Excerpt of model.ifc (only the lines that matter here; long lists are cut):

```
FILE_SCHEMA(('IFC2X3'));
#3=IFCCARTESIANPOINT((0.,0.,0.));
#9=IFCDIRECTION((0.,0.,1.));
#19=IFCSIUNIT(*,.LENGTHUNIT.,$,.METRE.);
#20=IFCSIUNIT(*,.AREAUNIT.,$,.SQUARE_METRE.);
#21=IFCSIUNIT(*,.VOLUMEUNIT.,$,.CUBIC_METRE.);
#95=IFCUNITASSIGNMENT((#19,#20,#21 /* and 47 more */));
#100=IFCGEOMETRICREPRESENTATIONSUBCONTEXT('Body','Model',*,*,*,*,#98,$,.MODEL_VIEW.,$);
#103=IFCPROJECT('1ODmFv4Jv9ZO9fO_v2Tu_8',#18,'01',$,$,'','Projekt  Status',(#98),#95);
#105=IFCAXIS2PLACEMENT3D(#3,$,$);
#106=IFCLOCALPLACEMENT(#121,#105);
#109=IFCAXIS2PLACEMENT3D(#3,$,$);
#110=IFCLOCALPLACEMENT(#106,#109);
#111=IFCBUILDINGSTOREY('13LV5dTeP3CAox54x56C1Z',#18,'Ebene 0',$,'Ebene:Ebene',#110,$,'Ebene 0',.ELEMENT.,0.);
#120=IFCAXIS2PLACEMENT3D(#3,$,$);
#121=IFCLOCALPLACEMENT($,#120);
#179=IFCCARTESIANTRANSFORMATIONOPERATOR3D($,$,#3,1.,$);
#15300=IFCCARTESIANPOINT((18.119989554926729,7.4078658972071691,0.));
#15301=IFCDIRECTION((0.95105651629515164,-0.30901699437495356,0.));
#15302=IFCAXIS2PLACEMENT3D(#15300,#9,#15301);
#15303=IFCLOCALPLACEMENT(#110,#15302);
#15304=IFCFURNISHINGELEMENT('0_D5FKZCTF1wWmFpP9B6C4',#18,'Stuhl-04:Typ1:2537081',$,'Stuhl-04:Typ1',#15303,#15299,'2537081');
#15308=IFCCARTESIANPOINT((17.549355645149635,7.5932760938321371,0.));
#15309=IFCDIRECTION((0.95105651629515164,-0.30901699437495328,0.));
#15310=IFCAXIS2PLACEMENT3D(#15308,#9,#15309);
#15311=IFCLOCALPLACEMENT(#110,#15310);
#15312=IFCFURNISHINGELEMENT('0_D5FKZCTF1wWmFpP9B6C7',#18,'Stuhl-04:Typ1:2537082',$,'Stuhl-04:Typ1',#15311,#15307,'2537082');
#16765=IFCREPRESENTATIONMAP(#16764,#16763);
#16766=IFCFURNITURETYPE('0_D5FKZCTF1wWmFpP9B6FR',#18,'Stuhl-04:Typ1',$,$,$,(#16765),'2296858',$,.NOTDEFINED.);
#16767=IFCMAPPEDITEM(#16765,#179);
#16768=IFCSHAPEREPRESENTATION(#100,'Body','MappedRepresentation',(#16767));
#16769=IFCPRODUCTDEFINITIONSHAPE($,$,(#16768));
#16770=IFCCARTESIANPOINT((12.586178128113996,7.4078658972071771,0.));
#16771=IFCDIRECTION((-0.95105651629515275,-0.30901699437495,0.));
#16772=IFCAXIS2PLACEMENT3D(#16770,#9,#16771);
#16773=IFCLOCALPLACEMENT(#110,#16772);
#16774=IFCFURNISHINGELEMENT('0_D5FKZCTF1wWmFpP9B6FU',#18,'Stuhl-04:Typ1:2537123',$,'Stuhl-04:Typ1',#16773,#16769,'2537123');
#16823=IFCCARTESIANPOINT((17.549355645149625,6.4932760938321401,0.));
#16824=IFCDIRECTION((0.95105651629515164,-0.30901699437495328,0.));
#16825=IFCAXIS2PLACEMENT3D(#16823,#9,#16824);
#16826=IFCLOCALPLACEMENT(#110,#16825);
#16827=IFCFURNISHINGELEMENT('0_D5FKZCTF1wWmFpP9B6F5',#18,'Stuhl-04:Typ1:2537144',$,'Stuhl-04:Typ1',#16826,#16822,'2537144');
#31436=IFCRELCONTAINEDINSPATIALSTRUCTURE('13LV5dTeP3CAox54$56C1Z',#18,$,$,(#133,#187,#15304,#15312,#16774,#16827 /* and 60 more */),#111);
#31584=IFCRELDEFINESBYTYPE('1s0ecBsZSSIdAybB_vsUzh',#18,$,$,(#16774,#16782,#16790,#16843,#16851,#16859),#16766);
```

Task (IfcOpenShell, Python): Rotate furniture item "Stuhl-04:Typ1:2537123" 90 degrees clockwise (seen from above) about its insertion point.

```python
import ifcopenshell
import ifcopenshell.api.geometry
import ifcopenshell.util.placement

model = ifcopenshell.open("model.ifc")

item = model.by_guid("0_D5FKZCTF1wWmFpP9B6FU")
matrix = ifcopenshell.util.placement.get_local_placement(item.ObjectPlacement)
matrix = matrix @ ifcopenshell.util.placement.rotation(-90, "Z")
ifcopenshell.api.geometry.edit_object_placement(model, product=item, matrix=matrix, is_si=False)

print(ifcopenshell.util.placement.get_local_placement(item.ObjectPlacement).round(3) + 0.0)

model.write("model_edited.ifc")
```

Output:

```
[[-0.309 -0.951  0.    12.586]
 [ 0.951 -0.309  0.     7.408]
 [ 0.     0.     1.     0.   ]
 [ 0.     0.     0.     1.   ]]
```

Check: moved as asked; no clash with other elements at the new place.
